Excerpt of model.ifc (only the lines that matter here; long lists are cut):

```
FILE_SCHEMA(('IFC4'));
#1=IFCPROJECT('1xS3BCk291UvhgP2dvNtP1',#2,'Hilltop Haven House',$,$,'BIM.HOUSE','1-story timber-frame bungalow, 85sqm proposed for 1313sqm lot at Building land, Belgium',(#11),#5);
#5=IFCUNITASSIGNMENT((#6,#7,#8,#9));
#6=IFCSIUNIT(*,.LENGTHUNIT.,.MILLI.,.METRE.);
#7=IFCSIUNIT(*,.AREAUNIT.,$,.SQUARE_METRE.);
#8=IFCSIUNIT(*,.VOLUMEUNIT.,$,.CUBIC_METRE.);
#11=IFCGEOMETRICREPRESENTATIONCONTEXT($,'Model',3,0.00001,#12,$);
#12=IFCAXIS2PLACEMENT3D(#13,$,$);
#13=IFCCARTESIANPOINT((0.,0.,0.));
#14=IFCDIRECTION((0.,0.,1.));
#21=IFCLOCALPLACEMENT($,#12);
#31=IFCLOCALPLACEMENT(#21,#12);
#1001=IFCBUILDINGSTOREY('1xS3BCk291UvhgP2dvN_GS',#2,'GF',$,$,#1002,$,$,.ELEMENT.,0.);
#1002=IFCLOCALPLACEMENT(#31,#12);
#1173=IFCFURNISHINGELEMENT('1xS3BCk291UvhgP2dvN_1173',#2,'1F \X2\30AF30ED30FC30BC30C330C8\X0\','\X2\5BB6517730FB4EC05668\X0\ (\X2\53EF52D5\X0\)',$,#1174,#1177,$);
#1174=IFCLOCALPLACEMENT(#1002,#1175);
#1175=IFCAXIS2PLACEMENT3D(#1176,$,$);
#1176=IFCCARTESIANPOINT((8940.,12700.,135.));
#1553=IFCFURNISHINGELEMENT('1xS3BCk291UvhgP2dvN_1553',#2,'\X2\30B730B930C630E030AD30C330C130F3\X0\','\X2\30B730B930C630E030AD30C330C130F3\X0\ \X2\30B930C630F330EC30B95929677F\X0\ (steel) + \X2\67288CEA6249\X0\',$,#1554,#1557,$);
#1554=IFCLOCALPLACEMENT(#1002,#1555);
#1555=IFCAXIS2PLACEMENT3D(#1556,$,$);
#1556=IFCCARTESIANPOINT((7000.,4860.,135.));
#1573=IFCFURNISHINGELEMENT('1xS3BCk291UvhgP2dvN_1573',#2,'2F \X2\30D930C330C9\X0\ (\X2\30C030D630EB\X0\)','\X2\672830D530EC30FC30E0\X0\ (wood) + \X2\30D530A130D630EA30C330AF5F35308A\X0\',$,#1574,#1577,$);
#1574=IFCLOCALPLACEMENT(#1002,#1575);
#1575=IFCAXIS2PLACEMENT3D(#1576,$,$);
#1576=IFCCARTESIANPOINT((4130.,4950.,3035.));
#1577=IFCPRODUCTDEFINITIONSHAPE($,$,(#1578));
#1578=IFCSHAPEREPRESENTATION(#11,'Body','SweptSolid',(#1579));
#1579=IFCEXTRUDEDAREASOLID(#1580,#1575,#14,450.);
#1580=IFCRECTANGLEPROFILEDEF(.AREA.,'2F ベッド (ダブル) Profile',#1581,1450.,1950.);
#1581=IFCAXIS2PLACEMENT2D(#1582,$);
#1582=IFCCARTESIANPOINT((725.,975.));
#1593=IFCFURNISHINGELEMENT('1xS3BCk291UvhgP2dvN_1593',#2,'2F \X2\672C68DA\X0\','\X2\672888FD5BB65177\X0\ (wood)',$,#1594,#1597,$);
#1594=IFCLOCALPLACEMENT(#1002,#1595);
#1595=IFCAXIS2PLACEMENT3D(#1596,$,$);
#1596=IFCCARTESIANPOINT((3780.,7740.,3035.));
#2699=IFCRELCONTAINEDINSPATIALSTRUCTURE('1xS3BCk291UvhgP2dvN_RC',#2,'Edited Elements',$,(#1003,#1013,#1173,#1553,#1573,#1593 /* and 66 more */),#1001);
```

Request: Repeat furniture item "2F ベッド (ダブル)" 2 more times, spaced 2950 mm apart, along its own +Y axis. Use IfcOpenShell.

```python
import ifcopenshell
import ifcopenshell.api.geometry
import ifcopenshell.api.root
import ifcopenshell.util.element
import ifcopenshell.util.placement
import ifcopenshell.util.unit

model = ifcopenshell.open("model.ifc")
unit_scale = ifcopenshell.util.unit.calculate_unit_scale(model)


def reuse_history(source, copy):
    """copy_class also copies each property set's owner history, people and application; keep the originals."""
    for rel in copy.IsDefinedBy:
        if rel.is_a("IfcRelDefinesByProperties") and (history := rel.RelatingPropertyDefinition.OwnerHistory):
            rel.RelatingPropertyDefinition.OwnerHistory = source.OwnerHistory
            ifcopenshell.util.element.remove_deep2(model, history)


source = model.by_guid("1xS3BCk291UvhgP2dvN_1573")
base = ifcopenshell.util.placement.get_local_placement(source.ObjectPlacement)
step = base[:3, 1] * 2.95 / unit_scale

for i in range(1, 3):
    copy = ifcopenshell.api.root.copy_class(model, product=source)
    copy.Representation = ifcopenshell.util.element.copy_deep(
        model, source.Representation, exclude=["IfcGeometricRepresentationContext", "IfcRepresentationMap"]
    )
    reuse_history(source, copy)
    matrix = base.copy()
    matrix[:3, 3] += i * step
    print("added at", matrix[:3, 3].round(3) + 0.0)
    ifcopenshell.api.geometry.edit_object_placement(model, product=copy, matrix=matrix, is_si=False)

model.write("model_v2.ifc")
```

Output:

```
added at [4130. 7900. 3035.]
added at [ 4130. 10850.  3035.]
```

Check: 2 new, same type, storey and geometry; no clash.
